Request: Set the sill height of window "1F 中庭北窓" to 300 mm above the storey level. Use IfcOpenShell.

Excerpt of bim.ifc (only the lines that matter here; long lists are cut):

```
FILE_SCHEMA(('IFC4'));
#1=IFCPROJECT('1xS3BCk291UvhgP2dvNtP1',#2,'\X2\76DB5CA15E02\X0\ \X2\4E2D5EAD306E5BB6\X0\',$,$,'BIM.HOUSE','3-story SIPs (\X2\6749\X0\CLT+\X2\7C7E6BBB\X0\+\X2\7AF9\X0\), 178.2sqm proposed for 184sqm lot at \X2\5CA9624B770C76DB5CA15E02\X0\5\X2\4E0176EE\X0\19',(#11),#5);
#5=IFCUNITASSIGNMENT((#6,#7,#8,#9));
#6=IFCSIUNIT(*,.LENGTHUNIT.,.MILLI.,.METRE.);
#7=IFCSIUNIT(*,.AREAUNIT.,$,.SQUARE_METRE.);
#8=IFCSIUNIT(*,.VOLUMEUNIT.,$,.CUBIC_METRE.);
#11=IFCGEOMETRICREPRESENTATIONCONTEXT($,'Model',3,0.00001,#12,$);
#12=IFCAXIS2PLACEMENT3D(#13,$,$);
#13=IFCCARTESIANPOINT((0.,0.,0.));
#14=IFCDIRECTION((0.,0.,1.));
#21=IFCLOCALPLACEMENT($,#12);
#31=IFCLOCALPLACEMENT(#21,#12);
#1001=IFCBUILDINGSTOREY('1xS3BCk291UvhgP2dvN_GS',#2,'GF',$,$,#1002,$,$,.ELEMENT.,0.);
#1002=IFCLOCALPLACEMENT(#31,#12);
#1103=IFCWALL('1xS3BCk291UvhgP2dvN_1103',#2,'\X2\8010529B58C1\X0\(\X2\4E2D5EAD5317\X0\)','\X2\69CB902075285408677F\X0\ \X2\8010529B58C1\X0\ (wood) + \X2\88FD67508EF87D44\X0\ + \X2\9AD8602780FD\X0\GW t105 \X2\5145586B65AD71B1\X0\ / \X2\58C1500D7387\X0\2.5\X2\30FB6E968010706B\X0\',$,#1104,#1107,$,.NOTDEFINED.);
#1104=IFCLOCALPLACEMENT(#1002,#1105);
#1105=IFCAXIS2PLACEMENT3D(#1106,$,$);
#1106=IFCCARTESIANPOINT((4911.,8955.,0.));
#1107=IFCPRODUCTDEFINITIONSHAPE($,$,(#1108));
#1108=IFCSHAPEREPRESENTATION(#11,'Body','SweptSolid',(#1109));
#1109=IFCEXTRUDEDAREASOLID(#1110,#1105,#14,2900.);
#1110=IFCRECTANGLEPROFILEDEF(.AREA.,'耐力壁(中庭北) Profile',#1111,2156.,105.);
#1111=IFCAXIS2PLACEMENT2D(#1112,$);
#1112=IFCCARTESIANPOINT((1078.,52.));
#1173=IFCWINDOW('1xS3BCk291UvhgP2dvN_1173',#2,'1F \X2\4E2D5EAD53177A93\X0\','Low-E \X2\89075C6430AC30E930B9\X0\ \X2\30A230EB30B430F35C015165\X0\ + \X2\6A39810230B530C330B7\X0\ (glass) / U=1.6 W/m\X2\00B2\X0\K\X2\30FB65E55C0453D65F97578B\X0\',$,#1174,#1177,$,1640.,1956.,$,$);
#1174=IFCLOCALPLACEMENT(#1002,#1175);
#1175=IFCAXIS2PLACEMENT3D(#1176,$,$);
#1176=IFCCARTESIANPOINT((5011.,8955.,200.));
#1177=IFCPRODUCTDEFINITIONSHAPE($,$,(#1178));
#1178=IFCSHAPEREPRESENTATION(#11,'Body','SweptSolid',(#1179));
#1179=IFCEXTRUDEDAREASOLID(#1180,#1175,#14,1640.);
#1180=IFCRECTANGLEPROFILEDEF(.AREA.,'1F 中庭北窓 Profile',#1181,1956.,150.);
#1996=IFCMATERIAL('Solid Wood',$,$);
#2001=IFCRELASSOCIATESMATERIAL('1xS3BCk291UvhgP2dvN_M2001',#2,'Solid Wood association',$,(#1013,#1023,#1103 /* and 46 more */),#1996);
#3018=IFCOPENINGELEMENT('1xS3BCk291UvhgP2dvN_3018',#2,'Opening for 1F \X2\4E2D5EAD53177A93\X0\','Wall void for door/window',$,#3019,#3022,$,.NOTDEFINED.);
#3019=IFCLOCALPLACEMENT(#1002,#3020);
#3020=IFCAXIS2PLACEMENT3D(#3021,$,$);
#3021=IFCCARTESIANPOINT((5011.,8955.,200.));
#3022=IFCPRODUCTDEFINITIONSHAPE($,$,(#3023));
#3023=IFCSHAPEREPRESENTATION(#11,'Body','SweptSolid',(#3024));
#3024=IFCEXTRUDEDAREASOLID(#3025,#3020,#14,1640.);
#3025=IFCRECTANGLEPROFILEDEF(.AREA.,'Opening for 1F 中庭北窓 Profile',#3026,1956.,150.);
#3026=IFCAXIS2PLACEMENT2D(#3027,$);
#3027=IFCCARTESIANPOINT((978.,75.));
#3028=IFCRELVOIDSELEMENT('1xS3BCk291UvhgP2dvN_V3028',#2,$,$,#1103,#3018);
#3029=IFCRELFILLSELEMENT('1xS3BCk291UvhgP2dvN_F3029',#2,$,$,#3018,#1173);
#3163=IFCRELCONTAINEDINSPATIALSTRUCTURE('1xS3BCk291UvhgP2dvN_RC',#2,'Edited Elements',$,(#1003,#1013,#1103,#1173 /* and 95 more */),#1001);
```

```python
import numpy as np
import ifcopenshell
import ifcopenshell.api.geometry
import ifcopenshell.geom
import ifcopenshell.util.element
import ifcopenshell.util.placement
import ifcopenshell.util.shape
import ifcopenshell.util.unit

model = ifcopenshell.open("bim.ifc")
unit_scale = ifcopenshell.util.unit.calculate_unit_scale(model)

window = model.by_guid("1xS3BCk291UvhgP2dvN_1173")
opening = window.FillsVoids[0].RelatingOpeningElement
storey = ifcopenshell.util.element.get_container(window, ifc_class="IfcBuildingStorey")
level = ifcopenshell.util.placement.get_local_placement(storey.ObjectPlacement)[2, 3]

# The opening's origin need not be at the sill, so measure its lowest point.
shape = ifcopenshell.geom.create_shape(ifcopenshell.geom.settings(), opening)
bottom = ifcopenshell.util.shape.get_shape_bottom_elevation(shape, shape.geometry) / unit_scale
dz = level + 0.3 / unit_scale - bottom

shift = np.array([0.0, 0.0, dz])
# The window is not placed relative to its opening, so move both.
for product in (opening, window):
    matrix = ifcopenshell.util.placement.get_local_placement(product.ObjectPlacement)
    matrix[:3, 3] += shift
    ifcopenshell.api.geometry.edit_object_placement(model, product=product, matrix=matrix, is_si=False)

print(f"moved by {dz * unit_scale:+.3f} m")

model.write("bim_v2.ifc")
```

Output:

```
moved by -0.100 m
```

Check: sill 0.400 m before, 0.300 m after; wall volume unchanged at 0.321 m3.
